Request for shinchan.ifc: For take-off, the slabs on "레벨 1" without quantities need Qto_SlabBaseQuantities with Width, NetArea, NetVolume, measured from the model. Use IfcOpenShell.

First a look at what the model holds.

```python
import ifcopenshell
import ifcopenshell.util.element
import ifcopenshell.util.unit

model = ifcopenshell.open("shinchan.ifc")
print(model.schema)
for unit_type in ("LENGTHUNIT", "AREAUNIT", "VOLUMEUNIT"):
    print(unit_type, ifcopenshell.util.unit.calculate_unit_scale(model, unit_type))
storey = next(s for s in model.by_type("IfcBuildingStorey") if s.Name == "레벨 1")
slabs = [e for e in ifcopenshell.util.element.get_decomposition(storey) if e.is_a("IfcSlab")]
for e in sorted(slabs, key=lambda e: e.id()):
    print(e.id(), e.is_a(), e.Name, list(ifcopenshell.util.element.get_psets(e, qtos_only=True)), sep=" | ")
```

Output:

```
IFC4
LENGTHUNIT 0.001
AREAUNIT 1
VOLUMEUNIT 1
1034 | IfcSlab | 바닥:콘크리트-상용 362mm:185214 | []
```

```python
import ifcopenshell
import ifcopenshell.api.pset
import ifcopenshell.geom
import ifcopenshell.util.element
import ifcopenshell.util.shape
import ifcopenshell.util.unit

model = ifcopenshell.open("shinchan.ifc")
unit_scale = ifcopenshell.util.unit.calculate_unit_scale(model)
area_scale = ifcopenshell.util.unit.calculate_unit_scale(model, "AREAUNIT")
volume_scale = ifcopenshell.util.unit.calculate_unit_scale(model, "VOLUMEUNIT")
settings = ifcopenshell.geom.settings()

storey = next(s for s in model.by_type("IfcBuildingStorey") if s.Name == "레벨 1")
slabs = [e for e in ifcopenshell.util.element.get_decomposition(storey) if e.is_a("IfcSlab")]

for e in sorted(slabs, key=lambda e: e.id()):
    if ifcopenshell.util.element.get_psets(e, qtos_only=True, should_inherit=False):
        continue
    # Geometry comes back in metres, in the element's own axes.
    shape = ifcopenshell.geom.create_shape(settings, e)
    values = {
        "Width": ifcopenshell.util.shape.get_z(shape.geometry) / unit_scale,
        "NetArea": ifcopenshell.util.shape.get_footprint_area(shape.geometry) / area_scale,
        "NetVolume": ifcopenshell.util.shape.get_volume(shape.geometry) / volume_scale,
    }
    qto = ifcopenshell.api.pset.add_qto(model, product=e, name="Qto_SlabBaseQuantities")
    ifcopenshell.api.pset.edit_qto(model, qto=qto, properties=values)
    print(e.id(), {k: round(v, 3) for k, v in values.items()})

model.write("shinchan-out.ifc")
```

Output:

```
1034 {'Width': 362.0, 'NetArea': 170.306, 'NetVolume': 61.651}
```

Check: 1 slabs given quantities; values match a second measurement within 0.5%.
